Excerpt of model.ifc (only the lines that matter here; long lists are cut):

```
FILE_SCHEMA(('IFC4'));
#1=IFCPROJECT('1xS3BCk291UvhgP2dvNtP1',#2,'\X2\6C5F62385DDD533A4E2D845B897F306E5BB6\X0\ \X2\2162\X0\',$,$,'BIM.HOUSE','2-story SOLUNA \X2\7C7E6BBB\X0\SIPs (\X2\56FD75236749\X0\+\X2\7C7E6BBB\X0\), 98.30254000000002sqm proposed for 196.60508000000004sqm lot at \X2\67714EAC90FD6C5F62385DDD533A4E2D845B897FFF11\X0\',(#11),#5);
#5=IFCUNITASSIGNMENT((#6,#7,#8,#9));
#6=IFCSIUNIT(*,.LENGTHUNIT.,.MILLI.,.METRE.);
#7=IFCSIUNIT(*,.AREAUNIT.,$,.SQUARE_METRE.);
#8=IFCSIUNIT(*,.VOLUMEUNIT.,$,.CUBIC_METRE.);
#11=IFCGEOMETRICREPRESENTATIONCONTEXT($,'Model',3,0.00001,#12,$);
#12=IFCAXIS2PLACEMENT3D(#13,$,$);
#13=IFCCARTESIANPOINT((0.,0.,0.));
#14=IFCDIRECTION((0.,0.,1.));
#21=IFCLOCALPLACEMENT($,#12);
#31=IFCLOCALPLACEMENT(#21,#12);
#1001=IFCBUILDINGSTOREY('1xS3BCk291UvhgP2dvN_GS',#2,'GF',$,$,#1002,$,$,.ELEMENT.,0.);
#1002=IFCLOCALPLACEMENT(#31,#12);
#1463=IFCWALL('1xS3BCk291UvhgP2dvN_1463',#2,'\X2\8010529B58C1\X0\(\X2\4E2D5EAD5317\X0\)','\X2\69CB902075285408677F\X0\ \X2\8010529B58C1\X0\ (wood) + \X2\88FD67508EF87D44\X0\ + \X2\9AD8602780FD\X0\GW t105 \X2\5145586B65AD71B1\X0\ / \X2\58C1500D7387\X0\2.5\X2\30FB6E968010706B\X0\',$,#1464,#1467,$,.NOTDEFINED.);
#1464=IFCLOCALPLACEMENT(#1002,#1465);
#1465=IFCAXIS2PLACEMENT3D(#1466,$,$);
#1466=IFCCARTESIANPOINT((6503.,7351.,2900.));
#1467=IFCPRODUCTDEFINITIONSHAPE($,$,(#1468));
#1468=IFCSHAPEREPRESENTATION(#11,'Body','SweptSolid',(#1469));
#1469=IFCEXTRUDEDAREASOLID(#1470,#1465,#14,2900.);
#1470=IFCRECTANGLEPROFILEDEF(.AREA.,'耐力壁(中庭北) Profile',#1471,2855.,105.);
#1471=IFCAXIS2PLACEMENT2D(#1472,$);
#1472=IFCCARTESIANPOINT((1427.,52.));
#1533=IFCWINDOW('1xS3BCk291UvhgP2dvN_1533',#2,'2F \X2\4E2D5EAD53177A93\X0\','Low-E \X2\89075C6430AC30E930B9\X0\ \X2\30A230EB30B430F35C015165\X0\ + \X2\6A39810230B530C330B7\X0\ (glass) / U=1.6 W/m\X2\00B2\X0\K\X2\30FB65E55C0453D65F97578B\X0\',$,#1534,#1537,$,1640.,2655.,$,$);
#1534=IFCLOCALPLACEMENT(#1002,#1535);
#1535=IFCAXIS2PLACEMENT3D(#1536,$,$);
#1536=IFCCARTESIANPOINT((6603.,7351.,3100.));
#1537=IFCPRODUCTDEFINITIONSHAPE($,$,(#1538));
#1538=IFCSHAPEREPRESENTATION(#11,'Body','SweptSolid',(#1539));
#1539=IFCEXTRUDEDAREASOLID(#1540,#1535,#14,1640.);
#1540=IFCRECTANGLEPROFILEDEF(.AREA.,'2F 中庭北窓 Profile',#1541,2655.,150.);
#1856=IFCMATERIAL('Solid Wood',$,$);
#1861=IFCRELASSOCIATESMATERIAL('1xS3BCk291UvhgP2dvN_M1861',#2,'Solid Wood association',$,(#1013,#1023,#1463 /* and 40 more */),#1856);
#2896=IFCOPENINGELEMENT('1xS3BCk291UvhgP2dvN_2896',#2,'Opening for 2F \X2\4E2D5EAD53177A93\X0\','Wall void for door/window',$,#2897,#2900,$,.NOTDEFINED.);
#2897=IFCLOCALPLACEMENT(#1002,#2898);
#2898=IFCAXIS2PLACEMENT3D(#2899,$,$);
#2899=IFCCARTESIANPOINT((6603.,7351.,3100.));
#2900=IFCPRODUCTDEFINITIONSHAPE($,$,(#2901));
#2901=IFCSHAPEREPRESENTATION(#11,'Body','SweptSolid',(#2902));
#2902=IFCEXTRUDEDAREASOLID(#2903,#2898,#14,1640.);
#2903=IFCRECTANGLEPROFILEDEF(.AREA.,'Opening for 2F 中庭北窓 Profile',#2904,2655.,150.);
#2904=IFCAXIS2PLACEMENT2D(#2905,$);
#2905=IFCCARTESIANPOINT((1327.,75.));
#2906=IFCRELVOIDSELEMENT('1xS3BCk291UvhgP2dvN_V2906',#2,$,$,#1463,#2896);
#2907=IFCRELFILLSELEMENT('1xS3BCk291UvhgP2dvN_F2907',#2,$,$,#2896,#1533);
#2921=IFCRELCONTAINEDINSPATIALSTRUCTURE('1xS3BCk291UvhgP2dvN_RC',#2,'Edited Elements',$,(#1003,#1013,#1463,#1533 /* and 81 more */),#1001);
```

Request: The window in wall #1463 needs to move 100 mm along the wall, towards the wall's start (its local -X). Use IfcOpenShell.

```python
import ifcopenshell
import ifcopenshell.api.geometry
import ifcopenshell.util.placement

model = ifcopenshell.open("model.ifc")

window = model.by_id(1533)
opening = window.FillsVoids[0].RelatingOpeningElement
wall = opening.VoidsElements[0].RelatingBuildingElement

wall_matrix = ifcopenshell.util.placement.get_local_placement(wall.ObjectPlacement)
shift = wall_matrix[:3, 0] * -100.0
before = ifcopenshell.util.placement.get_local_placement(window.ObjectPlacement)[:3, 3].copy()

# The window is not placed relative to its opening, so move both.
for product in (opening, window):
    matrix = ifcopenshell.util.placement.get_local_placement(product.ObjectPlacement)
    matrix[:3, 3] += shift
    ifcopenshell.api.geometry.edit_object_placement(model, product=product, matrix=matrix, is_si=False)

after = ifcopenshell.util.placement.get_local_placement(window.ObjectPlacement)[:3, 3]
print("window moved by", (after - before).round(3) + 0.0)

model.write("model_updated.ifc")
```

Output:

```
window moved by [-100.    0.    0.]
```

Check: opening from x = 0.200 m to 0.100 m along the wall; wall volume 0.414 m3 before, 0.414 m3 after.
